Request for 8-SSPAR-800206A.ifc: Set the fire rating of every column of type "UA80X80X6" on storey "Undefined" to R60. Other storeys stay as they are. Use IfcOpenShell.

First a look at what the model holds.

```python
import ifcopenshell
import ifcopenshell.util.element

model = ifcopenshell.open("8-SSPAR-800206A.ifc")
print(model.schema)
storey = next(s for s in model.by_type("IfcBuildingStorey") if s.Name == "Undefined")
columns = [e for e in ifcopenshell.util.element.get_decomposition(storey) if e.is_a("IfcColumn")]
seen = {}
for e in columns:
    element_type = ifcopenshell.util.element.get_type(e)
    key = (element_type.Name if element_type != e and element_type else None, ifcopenshell.util.element.get_pset(e, "Pset_ColumnCommon", "FireRating"))
    seen[key] = seen.get(key, 0) + 1
for (name, value), count in sorted(seen.items(), key=str):
    print(count, "x", name, "|", value)
```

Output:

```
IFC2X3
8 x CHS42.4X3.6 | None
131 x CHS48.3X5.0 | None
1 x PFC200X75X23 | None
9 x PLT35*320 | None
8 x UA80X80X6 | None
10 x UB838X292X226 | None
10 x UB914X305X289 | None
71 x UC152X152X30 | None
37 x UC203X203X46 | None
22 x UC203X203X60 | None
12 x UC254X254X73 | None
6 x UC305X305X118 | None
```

```python
import ifcopenshell
import ifcopenshell.api.pset
import ifcopenshell.util.element

model = ifcopenshell.open("8-SSPAR-800206A.ifc")

storey = next(s for s in model.by_type("IfcBuildingStorey") if s.Name == "Undefined")
columns = [e for e in ifcopenshell.util.element.get_decomposition(storey) if e.is_a("IfcColumn")]

count = 0
for e in columns:
    element_type = ifcopenshell.util.element.get_type(e)
    if element_type in (None, e) or element_type.Name != "UA80X80X6":
        continue
    # add_pset returns the element's existing set when there is one.
    pset = ifcopenshell.api.pset.add_pset(model, product=e, name="Pset_ColumnCommon")
    ifcopenshell.api.pset.edit_pset(model, pset=pset, properties={"FireRating": "R60"})
    count += 1

print(count, "columns updated")

model.write("8-SSPAR-800206A_rev.ifc")
```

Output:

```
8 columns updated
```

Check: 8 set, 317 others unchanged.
